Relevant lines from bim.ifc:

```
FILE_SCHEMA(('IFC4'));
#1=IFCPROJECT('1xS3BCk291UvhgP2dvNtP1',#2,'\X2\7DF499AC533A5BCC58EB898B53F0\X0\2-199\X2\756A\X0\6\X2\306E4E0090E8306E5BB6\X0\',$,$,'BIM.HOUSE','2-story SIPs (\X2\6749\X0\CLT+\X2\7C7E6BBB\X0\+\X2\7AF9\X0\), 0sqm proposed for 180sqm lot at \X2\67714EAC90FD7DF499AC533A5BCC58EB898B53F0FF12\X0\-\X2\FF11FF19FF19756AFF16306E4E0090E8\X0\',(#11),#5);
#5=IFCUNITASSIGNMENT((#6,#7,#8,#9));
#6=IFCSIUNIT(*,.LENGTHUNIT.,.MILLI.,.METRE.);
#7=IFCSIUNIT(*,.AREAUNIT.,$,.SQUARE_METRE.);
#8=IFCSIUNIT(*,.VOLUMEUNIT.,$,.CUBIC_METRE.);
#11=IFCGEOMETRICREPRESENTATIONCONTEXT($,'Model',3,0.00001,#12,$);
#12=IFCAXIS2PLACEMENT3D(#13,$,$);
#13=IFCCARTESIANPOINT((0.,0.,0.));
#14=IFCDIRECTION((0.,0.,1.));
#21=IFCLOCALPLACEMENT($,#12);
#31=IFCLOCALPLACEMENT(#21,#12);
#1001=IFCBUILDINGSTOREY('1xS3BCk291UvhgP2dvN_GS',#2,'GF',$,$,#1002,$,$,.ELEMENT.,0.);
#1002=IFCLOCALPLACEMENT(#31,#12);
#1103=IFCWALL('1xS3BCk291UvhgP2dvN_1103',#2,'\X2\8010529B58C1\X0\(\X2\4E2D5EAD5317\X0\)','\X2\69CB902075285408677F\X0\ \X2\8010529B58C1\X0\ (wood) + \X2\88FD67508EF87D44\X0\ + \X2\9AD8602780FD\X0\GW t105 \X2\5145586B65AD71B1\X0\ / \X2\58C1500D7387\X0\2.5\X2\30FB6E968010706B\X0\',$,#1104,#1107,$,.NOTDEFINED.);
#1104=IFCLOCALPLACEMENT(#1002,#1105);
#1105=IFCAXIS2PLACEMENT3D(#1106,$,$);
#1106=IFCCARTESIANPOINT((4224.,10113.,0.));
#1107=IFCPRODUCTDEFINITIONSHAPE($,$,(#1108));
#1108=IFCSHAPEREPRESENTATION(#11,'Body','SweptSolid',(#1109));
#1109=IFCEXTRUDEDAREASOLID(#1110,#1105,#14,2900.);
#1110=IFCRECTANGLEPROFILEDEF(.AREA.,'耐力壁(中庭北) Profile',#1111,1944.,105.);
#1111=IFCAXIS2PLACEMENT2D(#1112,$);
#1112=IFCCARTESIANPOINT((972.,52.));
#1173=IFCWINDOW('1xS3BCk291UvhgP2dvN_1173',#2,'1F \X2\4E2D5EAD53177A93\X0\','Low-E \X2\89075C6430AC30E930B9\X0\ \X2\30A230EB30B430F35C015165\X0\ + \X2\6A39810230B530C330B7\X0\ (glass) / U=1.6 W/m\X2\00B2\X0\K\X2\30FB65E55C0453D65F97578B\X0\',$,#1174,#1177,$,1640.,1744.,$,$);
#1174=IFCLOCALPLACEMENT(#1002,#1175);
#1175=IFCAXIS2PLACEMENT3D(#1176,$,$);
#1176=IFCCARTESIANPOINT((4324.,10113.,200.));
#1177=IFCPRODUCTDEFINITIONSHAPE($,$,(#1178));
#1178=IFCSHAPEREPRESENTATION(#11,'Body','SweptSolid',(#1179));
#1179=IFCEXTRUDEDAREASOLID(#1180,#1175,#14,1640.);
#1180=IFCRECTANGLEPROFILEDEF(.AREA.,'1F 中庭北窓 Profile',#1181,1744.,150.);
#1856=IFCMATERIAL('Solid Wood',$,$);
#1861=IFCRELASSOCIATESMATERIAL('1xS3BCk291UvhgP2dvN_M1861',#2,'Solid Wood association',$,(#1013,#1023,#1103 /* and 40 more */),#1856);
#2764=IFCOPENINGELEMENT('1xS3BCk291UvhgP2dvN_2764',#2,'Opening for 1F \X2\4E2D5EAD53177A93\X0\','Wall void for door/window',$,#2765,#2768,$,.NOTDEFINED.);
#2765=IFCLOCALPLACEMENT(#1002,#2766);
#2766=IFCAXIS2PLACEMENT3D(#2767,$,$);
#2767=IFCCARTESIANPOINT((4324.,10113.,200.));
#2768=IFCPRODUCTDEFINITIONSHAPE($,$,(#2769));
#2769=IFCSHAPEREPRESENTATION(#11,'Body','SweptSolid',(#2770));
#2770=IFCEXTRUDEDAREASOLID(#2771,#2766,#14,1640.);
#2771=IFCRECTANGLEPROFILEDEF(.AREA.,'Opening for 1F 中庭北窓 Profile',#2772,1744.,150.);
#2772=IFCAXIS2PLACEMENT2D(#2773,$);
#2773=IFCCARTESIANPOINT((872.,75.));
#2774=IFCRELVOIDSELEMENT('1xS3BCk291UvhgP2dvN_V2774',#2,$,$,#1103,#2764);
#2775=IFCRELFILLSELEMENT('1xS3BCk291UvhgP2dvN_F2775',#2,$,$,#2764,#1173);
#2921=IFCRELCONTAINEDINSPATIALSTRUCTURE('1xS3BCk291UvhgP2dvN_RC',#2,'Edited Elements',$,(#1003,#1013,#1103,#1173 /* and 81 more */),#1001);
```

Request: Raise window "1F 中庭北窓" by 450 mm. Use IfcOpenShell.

```python
import numpy as np
import ifcopenshell
import ifcopenshell.api.geometry
import ifcopenshell.util.placement
import ifcopenshell.util.unit

model = ifcopenshell.open("bim.ifc")
unit_scale = ifcopenshell.util.unit.calculate_unit_scale(model)

window = model.by_guid("1xS3BCk291UvhgP2dvN_1173")
opening = window.FillsVoids[0].RelatingOpeningElement
dz = 450.0

shift = np.array([0.0, 0.0, dz])
# The window is not placed relative to its opening, so move both.
for product in (opening, window):
    matrix = ifcopenshell.util.placement.get_local_placement(product.ObjectPlacement)
    matrix[:3, 3] += shift
    ifcopenshell.api.geometry.edit_object_placement(model, product=product, matrix=matrix, is_si=False)

print(f"moved by {dz * unit_scale:+.3f} m")

model.write("bim_edited.ifc")
```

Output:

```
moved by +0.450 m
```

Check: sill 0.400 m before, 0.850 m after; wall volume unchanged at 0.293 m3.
